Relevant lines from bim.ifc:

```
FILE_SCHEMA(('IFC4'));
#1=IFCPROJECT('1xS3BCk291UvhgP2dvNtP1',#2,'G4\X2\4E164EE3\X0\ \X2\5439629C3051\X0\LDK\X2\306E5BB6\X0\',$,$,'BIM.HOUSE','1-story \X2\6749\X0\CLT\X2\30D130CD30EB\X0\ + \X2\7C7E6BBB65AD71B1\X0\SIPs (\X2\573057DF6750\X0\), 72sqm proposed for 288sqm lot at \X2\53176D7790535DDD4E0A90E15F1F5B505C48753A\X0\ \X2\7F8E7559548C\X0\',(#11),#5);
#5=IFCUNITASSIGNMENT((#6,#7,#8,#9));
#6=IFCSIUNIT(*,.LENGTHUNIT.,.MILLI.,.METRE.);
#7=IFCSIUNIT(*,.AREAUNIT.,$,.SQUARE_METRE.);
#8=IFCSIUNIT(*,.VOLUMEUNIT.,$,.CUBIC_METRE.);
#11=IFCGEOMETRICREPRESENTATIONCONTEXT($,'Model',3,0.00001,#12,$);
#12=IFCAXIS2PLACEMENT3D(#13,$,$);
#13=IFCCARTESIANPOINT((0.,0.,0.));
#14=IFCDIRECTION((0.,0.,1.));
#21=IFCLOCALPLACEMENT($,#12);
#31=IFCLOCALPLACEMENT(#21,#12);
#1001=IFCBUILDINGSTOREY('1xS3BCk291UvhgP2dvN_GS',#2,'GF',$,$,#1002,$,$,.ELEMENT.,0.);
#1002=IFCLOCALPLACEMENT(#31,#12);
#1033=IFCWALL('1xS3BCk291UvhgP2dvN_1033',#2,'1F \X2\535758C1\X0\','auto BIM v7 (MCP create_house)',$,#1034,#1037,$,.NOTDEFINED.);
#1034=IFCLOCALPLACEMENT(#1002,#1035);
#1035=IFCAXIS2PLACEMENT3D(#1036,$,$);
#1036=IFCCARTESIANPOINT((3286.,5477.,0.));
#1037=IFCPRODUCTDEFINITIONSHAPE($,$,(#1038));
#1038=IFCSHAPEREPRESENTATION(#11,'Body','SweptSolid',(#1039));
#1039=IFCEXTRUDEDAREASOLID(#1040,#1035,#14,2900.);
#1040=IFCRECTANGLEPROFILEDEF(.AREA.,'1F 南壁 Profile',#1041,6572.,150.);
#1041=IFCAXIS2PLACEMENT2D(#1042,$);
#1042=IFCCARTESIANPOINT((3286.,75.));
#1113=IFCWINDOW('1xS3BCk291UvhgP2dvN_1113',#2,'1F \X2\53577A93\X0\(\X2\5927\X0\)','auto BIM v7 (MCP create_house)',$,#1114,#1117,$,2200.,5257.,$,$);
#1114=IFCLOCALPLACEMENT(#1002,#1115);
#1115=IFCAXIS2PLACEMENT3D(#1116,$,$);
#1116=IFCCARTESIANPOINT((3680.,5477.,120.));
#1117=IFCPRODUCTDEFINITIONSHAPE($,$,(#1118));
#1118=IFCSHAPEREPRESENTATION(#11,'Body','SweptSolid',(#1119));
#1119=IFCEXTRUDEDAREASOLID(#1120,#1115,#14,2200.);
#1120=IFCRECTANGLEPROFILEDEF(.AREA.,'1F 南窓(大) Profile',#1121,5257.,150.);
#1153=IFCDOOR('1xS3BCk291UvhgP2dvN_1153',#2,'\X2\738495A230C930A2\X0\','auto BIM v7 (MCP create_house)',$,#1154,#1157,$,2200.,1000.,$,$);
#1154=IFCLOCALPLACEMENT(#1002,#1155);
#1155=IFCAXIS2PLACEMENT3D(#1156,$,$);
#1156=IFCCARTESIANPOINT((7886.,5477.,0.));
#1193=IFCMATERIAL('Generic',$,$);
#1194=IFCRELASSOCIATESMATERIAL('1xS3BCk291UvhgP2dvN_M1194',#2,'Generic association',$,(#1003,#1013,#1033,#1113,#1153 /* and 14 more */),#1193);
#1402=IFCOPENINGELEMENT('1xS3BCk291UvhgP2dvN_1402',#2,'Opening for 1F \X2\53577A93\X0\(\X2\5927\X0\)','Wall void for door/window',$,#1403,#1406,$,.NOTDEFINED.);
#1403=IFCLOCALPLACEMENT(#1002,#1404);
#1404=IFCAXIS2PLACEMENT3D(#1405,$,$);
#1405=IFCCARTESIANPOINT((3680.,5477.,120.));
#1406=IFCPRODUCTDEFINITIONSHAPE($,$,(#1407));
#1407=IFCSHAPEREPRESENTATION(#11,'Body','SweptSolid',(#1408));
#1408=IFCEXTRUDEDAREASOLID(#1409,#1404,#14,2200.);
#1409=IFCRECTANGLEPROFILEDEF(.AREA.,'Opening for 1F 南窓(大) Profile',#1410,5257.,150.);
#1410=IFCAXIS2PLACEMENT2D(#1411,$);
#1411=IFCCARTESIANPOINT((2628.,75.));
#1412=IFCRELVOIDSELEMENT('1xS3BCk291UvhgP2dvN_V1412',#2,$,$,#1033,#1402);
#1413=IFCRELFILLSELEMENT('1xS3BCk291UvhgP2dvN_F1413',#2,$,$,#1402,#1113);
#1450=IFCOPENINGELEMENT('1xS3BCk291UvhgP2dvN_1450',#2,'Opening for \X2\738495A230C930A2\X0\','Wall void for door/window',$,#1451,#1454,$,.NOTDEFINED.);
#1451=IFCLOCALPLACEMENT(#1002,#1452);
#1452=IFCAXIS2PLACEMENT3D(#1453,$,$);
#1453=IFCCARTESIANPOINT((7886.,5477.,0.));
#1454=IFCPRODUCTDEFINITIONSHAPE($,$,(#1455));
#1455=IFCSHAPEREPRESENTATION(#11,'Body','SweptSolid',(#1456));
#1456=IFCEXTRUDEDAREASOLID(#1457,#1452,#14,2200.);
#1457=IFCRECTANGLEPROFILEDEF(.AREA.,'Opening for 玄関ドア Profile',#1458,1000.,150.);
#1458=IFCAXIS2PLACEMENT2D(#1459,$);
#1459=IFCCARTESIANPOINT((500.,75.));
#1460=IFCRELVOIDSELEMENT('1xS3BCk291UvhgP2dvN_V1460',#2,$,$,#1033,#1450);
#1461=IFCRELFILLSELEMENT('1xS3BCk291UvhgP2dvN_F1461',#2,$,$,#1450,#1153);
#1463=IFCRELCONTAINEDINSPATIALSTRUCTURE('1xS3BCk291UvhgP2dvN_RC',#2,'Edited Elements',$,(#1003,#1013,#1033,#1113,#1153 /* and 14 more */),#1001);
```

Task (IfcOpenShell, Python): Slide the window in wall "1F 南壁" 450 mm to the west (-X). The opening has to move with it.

```python
import ifcopenshell
import ifcopenshell.api.geometry
import ifcopenshell.util.placement
import ifcopenshell.util.unit

model = ifcopenshell.open("bim.ifc")
unit_scale = ifcopenshell.util.unit.calculate_unit_scale(model)

window = model.by_guid("1xS3BCk291UvhgP2dvN_1113")
opening = window.FillsVoids[0].RelatingOpeningElement
wall = opening.VoidsElements[0].RelatingBuildingElement

wall_matrix = ifcopenshell.util.placement.get_local_placement(wall.ObjectPlacement)
shift = wall_matrix[:3, 0] * -0.45 / unit_scale
before = ifcopenshell.util.placement.get_local_placement(window.ObjectPlacement)[:3, 3].copy()

# The window is not placed relative to its opening, so move both.
for product in (opening, window):
    matrix = ifcopenshell.util.placement.get_local_placement(product.ObjectPlacement)
    matrix[:3, 3] += shift
    ifcopenshell.api.geometry.edit_object_placement(model, product=product, matrix=matrix, is_si=False)

after = ifcopenshell.util.placement.get_local_placement(window.ObjectPlacement)[:3, 3]
print("window moved by", (after - before).round(3) + 0.0)

model.write("bim-out.ifc")
```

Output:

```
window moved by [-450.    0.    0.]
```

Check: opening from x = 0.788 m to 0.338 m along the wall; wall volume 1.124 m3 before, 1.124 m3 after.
